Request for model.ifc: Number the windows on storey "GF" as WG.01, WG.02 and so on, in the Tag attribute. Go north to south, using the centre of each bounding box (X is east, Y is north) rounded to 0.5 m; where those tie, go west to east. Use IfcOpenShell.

First a look at what the model holds.

```python
import ifcopenshell
import ifcopenshell.util.element
import ifcopenshell.util.placement

model = ifcopenshell.open("model.ifc")
print(model.schema)
storey = next(s for s in model.by_type("IfcBuildingStorey") if s.Name == "GF")
windows = [e for e in ifcopenshell.util.element.get_decomposition(storey) if e.is_a("IfcWindow")]
for e in sorted(windows, key=lambda e: e.id()):
    origin = ifcopenshell.util.placement.get_local_placement(e.ObjectPlacement)[:3, 3]
    print(e.id(), e.Tag, e.Name, origin.round(2) + 0.0, sep=" | ")
```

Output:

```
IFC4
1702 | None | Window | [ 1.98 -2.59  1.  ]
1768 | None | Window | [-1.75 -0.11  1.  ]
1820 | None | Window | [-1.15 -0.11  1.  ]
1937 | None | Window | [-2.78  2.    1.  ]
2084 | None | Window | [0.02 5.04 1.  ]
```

```python
import ifcopenshell
import ifcopenshell.geom
import ifcopenshell.util.element
import ifcopenshell.util.shape

model = ifcopenshell.open("model.ifc")
settings = ifcopenshell.geom.settings()
settings.set("use-world-coords", True)


def centre(element):
    shape = ifcopenshell.geom.create_shape(settings, element)
    return ifcopenshell.util.shape.get_bbox_centroid(shape.geometry)


storey = next(s for s in model.by_type("IfcBuildingStorey") if s.Name == "GF")
windows = [e for e in ifcopenshell.util.element.get_decomposition(storey) if e.is_a("IfcWindow")]

# Insertion points can sit at a corner or the storey origin, so sort by the geometry (in metres).
centres = {e: centre(e) for e in windows}
windows.sort(key=lambda e: (-round(centres[e][1] / 0.5), centres[e][0]))

for i, e in enumerate(windows, start=1):
    number = f"WG.{i:02d}"
    e.Tag = number
    print(e.id(), number)

model.write("model_v2.ifc")
```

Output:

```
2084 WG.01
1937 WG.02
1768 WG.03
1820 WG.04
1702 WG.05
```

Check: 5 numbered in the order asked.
